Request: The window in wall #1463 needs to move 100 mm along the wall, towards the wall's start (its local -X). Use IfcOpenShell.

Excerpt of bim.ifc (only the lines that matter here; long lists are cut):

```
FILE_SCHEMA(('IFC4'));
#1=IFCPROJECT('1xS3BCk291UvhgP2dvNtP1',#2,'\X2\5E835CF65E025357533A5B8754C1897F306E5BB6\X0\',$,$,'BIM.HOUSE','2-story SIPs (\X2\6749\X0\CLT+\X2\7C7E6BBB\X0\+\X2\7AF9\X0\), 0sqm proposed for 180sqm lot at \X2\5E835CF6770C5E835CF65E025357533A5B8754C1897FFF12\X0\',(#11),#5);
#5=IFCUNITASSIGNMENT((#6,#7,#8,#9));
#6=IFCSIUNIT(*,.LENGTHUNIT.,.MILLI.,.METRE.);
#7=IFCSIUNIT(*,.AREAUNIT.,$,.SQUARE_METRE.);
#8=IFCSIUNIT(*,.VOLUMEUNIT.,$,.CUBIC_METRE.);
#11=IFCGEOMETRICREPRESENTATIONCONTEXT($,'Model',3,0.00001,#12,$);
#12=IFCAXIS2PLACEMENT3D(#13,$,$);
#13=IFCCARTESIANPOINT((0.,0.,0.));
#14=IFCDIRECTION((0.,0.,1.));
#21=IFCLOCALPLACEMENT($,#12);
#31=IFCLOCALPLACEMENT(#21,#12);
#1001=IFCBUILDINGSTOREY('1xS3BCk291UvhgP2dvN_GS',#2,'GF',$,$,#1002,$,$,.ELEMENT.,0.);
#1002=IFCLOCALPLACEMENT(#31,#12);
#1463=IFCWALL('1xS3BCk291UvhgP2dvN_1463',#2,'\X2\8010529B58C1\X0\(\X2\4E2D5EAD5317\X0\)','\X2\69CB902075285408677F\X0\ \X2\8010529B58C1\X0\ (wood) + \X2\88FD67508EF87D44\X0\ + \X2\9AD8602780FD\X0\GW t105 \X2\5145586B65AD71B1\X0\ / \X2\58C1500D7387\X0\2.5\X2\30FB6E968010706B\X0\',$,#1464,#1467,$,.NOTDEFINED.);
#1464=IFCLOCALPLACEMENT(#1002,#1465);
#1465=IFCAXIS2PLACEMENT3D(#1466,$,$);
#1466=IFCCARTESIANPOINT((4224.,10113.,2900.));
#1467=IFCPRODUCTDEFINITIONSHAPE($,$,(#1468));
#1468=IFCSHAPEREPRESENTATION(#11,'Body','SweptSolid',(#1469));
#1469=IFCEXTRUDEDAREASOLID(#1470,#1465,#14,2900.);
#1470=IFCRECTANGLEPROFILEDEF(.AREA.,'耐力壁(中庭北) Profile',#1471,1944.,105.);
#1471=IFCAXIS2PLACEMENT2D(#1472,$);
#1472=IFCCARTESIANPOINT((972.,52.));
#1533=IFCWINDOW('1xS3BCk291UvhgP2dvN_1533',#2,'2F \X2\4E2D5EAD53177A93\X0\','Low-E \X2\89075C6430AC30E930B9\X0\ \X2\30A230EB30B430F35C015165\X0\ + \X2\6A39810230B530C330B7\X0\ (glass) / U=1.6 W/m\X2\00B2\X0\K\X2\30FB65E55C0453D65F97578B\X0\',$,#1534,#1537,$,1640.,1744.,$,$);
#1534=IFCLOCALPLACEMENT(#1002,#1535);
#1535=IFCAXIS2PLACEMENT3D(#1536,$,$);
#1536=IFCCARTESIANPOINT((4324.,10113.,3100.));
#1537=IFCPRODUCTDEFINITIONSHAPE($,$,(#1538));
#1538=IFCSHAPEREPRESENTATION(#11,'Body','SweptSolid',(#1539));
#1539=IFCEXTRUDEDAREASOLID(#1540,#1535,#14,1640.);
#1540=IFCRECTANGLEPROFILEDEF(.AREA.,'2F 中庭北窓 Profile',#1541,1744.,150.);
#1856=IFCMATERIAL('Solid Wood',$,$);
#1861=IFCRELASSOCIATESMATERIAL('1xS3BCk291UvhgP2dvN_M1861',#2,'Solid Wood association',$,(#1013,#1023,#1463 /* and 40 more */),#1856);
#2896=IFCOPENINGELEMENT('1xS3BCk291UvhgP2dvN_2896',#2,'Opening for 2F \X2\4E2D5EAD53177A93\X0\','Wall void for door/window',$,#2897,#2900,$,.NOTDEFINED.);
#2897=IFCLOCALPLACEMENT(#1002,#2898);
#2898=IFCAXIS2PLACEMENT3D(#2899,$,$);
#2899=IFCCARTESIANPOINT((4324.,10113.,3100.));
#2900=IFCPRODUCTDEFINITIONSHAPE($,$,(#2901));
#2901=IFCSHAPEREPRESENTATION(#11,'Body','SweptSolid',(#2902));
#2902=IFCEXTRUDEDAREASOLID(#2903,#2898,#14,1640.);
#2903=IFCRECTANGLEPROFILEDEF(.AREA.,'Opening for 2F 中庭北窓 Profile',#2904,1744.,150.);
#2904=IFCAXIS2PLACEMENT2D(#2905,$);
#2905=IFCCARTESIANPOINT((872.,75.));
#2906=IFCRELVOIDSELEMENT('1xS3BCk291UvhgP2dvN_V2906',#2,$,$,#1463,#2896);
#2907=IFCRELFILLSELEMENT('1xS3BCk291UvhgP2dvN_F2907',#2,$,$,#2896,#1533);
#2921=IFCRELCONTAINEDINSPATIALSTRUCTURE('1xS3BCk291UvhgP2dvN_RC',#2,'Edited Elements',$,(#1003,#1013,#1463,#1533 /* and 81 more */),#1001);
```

```python
import ifcopenshell
import ifcopenshell.api.geometry
import ifcopenshell.util.placement
import ifcopenshell.util.unit

model = ifcopenshell.open("bim.ifc")
unit_scale = ifcopenshell.util.unit.calculate_unit_scale(model)

window = model.by_id(1533)
opening = window.FillsVoids[0].RelatingOpeningElement
wall = opening.VoidsElements[0].RelatingBuildingElement

wall_matrix = ifcopenshell.util.placement.get_local_placement(wall.ObjectPlacement)
shift = wall_matrix[:3, 0] * -0.1 / unit_scale
before = ifcopenshell.util.placement.get_local_placement(window.ObjectPlacement)[:3, 3].copy()

# The window is not placed relative to its opening, so move both.
for product in (opening, window):
    matrix = ifcopenshell.util.placement.get_local_placement(product.ObjectPlacement)
    matrix[:3, 3] += shift
    ifcopenshell.api.geometry.edit_object_placement(model, product=product, matrix=matrix, is_si=False)

after = ifcopenshell.util.placement.get_local_placement(window.ObjectPlacement)[:3, 3]
print("window moved by", (after - before).round(3) + 0.0)

model.write("bim_updated.ifc")
```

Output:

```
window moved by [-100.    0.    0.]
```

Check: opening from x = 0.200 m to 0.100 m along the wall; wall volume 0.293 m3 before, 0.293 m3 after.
